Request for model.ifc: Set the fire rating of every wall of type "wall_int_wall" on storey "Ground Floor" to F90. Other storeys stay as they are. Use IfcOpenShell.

First a look at what the model holds.

```python
import ifcopenshell
import ifcopenshell.util.element

model = ifcopenshell.open("model.ifc")
print(model.schema)
storey = next(s for s in model.by_type("IfcBuildingStorey") if s.Name == "Ground Floor")
walls = [e for e in ifcopenshell.util.element.get_decomposition(storey) if e.is_a("IfcWall")]
seen = {}
for e in walls:
    element_type = ifcopenshell.util.element.get_type(e)
    key = (element_type.Name if element_type != e and element_type else None, ifcopenshell.util.element.get_pset(e, "Pset_WallCommon", "FireRating"))
    seen[key] = seen.get(key, 0) + 1
for (name, value), count in sorted(seen.items(), key=str):
    print(count, "x", name, "|", value)
```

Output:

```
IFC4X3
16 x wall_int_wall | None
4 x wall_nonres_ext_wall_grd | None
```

```python
import ifcopenshell
import ifcopenshell.api.pset
import ifcopenshell.util.element

model = ifcopenshell.open("model.ifc")

storey = next(s for s in model.by_type("IfcBuildingStorey") if s.Name == "Ground Floor")
walls = [e for e in ifcopenshell.util.element.get_decomposition(storey) if e.is_a("IfcWall")]

count = 0
for e in walls:
    element_type = ifcopenshell.util.element.get_type(e)
    if element_type in (None, e) or element_type.Name != "wall_int_wall":
        continue
    # add_pset returns the element's existing set when there is one.
    pset = ifcopenshell.api.pset.add_pset(model, product=e, name="Pset_WallCommon")
    ifcopenshell.api.pset.edit_pset(model, pset=pset, properties={"FireRating": "F90"})
    count += 1

print(count, "walls updated")

model.write("model_v2.ifc")
```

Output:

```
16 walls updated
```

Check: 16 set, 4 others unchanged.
